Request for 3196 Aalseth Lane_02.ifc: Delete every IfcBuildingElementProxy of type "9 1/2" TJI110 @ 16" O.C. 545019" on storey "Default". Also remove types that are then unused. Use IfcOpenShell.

First a look at what the model holds.

```python
import ifcopenshell
import ifcopenshell.util.element

model = ifcopenshell.open("3196 Aalseth Lane_02.ifc")
print(model.schema)
storey = next(s for s in model.by_type("IfcBuildingStorey") if s.Name == "Default")
proxies = [e for e in ifcopenshell.util.element.get_decomposition(storey) if e.is_a("IfcBuildingElementProxy")]
seen = {}
for e in proxies:
    element_type = ifcopenshell.util.element.get_type(e)
    name = element_type.Name if element_type not in (None, e) else None
    seen[name] = seen.get(name, 0) + 1
for name, count in sorted(seen.items(), key=str):
    print(count, "x", name)
```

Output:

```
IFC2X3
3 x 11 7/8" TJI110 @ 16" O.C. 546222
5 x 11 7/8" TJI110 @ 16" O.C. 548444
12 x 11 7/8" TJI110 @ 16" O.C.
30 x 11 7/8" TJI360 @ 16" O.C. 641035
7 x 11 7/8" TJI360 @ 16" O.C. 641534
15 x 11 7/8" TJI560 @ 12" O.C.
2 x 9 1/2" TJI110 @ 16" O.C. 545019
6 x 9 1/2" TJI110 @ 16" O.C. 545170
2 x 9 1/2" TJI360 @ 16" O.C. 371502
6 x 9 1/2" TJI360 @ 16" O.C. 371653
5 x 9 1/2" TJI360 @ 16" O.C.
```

```python
import ifcopenshell
import ifcopenshell.api.root
import ifcopenshell.util.element

model = ifcopenshell.open("3196 Aalseth Lane_02.ifc")

storey = next(s for s in model.by_type("IfcBuildingStorey") if s.Name == "Default")
proxies = [e for e in ifcopenshell.util.element.get_decomposition(storey) if e.is_a("IfcBuildingElementProxy")]
targets = [e for e in proxies if (t := ifcopenshell.util.element.get_type(e)) not in (None, e) and t.Name == '9 1/2" TJI110 @ 16" O.C. 545019']
types = {ifcopenshell.util.element.get_type(e) for e in targets} - {None, *targets}

for e in targets:
    ifcopenshell.api.root.remove_product(model, product=e)
print(len(targets), "removed")

unused = [t for t in types if not ifcopenshell.util.element.get_types(t)]
for t in unused:
    ifcopenshell.api.root.remove_product(model, product=t)
print(len(unused), "unused types removed")

model.write("3196 Aalseth Lane_02_v2.ifc")
```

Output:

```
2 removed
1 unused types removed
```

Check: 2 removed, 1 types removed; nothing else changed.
